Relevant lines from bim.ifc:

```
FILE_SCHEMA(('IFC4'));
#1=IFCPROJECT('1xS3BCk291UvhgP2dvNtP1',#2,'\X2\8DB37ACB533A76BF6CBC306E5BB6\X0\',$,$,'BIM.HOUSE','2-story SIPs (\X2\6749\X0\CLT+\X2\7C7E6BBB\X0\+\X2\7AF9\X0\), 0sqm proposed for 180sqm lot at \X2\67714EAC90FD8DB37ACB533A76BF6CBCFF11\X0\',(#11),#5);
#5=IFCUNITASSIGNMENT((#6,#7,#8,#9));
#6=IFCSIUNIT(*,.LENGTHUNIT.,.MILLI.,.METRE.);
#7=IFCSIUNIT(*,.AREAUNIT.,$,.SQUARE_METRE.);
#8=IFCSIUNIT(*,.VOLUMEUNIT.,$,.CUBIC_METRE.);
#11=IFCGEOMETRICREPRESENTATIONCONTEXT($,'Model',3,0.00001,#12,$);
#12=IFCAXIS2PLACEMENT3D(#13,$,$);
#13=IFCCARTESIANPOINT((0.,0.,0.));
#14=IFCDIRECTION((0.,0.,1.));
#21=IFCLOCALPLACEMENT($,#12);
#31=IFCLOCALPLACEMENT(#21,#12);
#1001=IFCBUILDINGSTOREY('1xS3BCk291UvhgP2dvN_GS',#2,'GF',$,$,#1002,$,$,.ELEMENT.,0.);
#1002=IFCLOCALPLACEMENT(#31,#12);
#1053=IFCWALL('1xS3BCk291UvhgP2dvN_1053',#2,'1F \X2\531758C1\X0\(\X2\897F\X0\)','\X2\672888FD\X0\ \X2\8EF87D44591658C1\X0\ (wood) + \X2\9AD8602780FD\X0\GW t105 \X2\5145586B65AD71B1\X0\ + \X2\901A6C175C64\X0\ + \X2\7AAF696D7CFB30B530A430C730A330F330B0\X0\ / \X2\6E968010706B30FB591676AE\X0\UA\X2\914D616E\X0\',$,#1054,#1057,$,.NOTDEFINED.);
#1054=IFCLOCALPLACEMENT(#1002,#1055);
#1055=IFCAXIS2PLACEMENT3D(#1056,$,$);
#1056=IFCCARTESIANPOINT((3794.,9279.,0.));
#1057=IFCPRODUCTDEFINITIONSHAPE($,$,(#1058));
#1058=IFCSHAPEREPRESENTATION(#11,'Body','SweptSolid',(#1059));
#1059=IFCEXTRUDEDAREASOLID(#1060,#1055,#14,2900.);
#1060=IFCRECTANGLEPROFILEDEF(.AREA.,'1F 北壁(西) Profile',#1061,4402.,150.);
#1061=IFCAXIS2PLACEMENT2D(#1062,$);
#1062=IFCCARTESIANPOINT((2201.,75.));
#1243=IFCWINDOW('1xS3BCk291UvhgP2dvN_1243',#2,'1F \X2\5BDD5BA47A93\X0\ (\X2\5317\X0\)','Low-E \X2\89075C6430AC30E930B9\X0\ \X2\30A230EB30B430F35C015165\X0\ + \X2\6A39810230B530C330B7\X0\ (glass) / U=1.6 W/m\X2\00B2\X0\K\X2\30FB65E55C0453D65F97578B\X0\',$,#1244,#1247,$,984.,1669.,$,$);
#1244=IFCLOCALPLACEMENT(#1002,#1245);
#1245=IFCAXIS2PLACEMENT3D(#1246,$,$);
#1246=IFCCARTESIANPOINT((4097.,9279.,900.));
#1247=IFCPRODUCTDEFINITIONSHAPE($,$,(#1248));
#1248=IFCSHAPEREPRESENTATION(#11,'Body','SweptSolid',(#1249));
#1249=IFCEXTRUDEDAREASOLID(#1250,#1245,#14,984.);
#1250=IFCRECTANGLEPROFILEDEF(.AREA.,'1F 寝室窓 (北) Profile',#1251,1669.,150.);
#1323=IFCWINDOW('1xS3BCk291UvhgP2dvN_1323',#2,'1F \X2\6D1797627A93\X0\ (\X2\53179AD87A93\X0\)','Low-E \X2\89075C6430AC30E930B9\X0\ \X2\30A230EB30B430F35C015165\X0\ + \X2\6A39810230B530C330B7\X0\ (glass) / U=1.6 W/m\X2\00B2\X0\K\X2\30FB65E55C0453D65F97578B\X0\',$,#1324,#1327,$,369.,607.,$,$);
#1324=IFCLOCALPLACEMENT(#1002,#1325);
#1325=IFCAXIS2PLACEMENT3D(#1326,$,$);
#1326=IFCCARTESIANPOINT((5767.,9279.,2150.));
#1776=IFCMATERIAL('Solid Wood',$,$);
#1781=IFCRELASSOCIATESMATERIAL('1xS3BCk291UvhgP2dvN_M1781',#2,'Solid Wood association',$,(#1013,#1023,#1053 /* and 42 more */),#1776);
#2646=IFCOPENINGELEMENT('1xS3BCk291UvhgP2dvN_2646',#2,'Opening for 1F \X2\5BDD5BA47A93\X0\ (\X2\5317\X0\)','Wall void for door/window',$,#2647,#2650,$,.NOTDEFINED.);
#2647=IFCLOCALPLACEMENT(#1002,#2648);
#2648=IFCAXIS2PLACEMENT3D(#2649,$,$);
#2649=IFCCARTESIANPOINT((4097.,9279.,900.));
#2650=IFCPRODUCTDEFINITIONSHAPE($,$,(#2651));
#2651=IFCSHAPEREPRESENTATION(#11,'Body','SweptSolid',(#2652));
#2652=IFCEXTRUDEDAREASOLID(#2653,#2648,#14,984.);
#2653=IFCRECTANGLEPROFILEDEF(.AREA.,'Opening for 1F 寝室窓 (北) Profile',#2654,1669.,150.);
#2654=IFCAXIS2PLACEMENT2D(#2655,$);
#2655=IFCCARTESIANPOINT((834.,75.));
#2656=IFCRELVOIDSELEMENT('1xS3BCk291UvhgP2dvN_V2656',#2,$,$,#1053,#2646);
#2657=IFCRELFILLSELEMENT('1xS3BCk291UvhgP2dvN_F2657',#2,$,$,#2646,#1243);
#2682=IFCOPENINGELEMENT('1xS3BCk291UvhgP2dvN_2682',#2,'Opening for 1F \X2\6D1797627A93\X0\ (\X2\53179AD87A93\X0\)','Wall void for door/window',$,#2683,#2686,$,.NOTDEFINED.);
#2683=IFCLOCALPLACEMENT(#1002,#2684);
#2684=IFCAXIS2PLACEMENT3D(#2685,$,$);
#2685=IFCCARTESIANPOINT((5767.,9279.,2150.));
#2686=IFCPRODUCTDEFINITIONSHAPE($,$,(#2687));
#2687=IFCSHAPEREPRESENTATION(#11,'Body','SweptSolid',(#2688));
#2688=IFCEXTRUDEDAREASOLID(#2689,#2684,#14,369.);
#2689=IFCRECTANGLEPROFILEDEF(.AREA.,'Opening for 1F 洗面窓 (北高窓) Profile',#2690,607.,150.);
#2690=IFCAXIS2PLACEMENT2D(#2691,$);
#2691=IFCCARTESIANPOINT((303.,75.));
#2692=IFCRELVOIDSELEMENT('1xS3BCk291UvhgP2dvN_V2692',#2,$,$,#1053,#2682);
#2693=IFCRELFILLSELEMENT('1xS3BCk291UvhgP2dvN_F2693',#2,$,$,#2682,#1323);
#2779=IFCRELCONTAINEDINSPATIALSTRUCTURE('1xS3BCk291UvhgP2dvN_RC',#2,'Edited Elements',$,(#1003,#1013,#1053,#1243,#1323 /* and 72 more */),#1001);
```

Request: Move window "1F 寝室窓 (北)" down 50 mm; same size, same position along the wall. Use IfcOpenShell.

```python
import numpy as np
import ifcopenshell
import ifcopenshell.api.geometry
import ifcopenshell.util.placement
import ifcopenshell.util.unit

model = ifcopenshell.open("bim.ifc")
unit_scale = ifcopenshell.util.unit.calculate_unit_scale(model)

window = model.by_guid("1xS3BCk291UvhgP2dvN_1243")
opening = window.FillsVoids[0].RelatingOpeningElement
dz = -0.05 / unit_scale

shift = np.array([0.0, 0.0, dz])
# The window is not placed relative to its opening, so move both.
for product in (opening, window):
    matrix = ifcopenshell.util.placement.get_local_placement(product.ObjectPlacement)
    matrix[:3, 3] += shift
    ifcopenshell.api.geometry.edit_object_placement(model, product=product, matrix=matrix, is_si=False)

print(f"moved by {dz * unit_scale:+.3f} m")

model.write("bim_rev.ifc")
```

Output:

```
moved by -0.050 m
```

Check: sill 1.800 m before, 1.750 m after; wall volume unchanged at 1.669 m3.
